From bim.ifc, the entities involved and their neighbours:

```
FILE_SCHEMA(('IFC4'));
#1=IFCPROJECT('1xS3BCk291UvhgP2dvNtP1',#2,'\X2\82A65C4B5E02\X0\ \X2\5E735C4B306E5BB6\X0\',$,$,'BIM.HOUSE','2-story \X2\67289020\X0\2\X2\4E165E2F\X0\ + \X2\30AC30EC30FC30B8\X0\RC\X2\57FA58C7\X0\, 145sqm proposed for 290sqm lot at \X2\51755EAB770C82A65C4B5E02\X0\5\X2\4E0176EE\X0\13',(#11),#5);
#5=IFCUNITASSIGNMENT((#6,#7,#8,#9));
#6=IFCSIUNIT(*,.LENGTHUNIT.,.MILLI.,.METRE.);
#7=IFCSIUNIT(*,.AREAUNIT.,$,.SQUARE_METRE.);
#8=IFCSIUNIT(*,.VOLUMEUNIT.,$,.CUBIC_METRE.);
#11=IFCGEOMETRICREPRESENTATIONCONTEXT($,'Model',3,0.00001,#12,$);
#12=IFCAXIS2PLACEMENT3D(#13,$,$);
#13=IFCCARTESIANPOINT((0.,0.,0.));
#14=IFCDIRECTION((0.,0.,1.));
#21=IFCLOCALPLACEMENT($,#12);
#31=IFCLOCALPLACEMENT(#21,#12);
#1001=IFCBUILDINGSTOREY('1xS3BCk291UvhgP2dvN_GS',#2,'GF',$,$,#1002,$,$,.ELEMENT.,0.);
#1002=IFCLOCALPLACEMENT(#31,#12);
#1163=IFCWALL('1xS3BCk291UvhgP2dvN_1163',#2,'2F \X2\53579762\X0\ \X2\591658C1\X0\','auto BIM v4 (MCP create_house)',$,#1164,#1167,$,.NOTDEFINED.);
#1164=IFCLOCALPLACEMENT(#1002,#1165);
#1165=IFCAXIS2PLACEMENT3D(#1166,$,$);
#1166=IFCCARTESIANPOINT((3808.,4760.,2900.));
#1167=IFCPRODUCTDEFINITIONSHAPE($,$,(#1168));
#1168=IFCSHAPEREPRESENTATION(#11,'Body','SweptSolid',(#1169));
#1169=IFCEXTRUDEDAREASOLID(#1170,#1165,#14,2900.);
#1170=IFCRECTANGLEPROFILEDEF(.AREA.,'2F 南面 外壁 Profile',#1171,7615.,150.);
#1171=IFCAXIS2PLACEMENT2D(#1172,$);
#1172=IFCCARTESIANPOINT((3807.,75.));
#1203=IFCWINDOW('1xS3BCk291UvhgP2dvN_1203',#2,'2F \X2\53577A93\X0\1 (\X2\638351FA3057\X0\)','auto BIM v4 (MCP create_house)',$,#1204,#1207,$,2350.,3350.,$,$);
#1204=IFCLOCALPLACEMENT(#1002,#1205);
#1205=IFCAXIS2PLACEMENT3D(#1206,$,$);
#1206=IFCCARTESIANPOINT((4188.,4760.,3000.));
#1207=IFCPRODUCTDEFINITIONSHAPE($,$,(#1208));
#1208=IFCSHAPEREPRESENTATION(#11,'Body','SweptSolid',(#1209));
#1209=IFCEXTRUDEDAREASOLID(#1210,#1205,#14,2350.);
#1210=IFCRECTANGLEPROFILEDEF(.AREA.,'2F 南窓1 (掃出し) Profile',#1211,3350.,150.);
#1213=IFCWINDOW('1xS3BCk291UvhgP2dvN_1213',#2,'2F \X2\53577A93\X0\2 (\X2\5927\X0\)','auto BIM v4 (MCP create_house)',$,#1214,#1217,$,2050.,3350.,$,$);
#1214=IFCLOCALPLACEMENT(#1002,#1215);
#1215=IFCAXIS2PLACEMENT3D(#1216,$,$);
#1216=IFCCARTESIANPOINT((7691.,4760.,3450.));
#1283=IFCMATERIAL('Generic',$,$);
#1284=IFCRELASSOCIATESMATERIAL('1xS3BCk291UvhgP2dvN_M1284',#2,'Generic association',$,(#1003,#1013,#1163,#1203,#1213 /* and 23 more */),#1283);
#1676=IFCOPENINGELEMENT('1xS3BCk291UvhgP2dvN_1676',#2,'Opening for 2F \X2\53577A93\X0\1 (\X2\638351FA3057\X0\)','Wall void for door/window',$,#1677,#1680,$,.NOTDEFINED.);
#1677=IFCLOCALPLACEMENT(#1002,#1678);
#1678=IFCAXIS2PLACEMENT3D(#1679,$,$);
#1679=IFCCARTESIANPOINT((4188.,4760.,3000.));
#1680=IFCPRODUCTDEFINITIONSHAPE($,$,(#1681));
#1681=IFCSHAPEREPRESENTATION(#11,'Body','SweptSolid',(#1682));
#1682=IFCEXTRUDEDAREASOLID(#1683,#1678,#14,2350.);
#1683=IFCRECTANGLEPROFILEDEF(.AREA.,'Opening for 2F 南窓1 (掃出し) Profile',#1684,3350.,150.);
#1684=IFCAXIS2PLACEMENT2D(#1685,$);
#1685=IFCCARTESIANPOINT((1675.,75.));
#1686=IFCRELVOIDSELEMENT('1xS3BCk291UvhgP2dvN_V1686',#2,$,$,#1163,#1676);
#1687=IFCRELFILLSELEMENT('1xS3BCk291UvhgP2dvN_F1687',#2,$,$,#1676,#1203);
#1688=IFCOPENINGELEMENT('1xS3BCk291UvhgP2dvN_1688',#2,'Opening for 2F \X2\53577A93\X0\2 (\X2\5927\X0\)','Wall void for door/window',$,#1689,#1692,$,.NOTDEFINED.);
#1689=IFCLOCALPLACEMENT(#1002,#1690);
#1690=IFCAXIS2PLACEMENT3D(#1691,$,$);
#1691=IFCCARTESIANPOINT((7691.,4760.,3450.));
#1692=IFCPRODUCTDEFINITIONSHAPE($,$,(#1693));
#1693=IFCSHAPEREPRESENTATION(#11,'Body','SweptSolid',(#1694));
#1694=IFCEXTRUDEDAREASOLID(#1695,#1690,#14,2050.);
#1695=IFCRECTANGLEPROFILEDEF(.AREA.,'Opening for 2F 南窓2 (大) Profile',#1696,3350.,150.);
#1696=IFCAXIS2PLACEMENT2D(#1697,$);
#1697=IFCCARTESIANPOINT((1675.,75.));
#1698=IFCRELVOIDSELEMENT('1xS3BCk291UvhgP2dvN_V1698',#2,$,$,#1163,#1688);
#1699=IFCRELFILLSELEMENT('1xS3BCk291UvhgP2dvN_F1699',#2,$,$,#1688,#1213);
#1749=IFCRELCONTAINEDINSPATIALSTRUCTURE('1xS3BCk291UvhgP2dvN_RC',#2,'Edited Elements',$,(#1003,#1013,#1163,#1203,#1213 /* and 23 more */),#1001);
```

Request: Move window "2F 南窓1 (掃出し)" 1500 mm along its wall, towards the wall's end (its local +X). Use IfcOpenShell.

```python
import ifcopenshell
import ifcopenshell.api.geometry
import ifcopenshell.util.placement

model = ifcopenshell.open("bim.ifc")

window = model.by_id(1203)
opening = window.FillsVoids[0].RelatingOpeningElement
wall = opening.VoidsElements[0].RelatingBuildingElement

wall_matrix = ifcopenshell.util.placement.get_local_placement(wall.ObjectPlacement)
shift = wall_matrix[:3, 0] * 1500.0
before = ifcopenshell.util.placement.get_local_placement(window.ObjectPlacement)[:3, 3].copy()

# The window is not placed relative to its opening, so move both.
for product in (opening, window):
    matrix = ifcopenshell.util.placement.get_local_placement(product.ObjectPlacement)
    matrix[:3, 3] += shift
    ifcopenshell.api.geometry.edit_object_placement(model, product=product, matrix=matrix, is_si=False)

after = ifcopenshell.util.placement.get_local_placement(window.ObjectPlacement)[:3, 3]
print("window moved by", (after - before).round(3) + 0.0)

model.write("bim-out.ifc")
```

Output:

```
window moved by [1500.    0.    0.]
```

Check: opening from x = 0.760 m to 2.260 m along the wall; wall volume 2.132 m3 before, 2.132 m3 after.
